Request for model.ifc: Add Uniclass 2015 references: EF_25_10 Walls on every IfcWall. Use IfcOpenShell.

First a look at what the model holds.

```python
import ifcopenshell

model = ifcopenshell.open("model.ifc")
print(model.schema)
print("classifications:", [c.Name for c in model.by_type("IfcClassification")])
for ifc_class in ("IfcDoor", "IfcRoof", "IfcStair", "IfcWall", "IfcWindow"):
    print(ifc_class, len(model.by_type(ifc_class)))
```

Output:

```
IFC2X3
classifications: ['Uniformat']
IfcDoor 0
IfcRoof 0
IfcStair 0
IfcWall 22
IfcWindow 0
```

```python
import ifcopenshell
import ifcopenshell.api.classification

model = ifcopenshell.open("model.ifc")

# IFC2X3 requires Source and Edition and has no link from the project to the system.
system = model.create_entity("IfcClassification", Source="NBS", Edition="2015", Name="Uniclass 2015")

codes = {
    "IfcWall": ("EF_25_10", "Walls"),
}
for ifc_class, (code, name) in codes.items():
    products = model.by_type(ifc_class)
    ifcopenshell.api.classification.add_reference(
        model, products=products, classification=system, identification=code, name=name
    )
    print(code, len(products))

model.write("model_v2.ifc")
```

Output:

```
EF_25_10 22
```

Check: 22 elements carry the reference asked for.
